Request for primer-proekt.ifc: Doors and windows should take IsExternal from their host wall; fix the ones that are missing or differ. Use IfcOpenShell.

First a look at what the model holds.

```python
import ifcopenshell
import ifcopenshell.util.element

model = ifcopenshell.open("primer-proekt.ifc")
print(model.schema)
seen = {}
for e in model.by_type("IfcDoor") + model.by_type("IfcWindow"):
    if not e.FillsVoids:
        continue
    host = e.FillsVoids[0].RelatingOpeningElement.VoidsElements[0].RelatingBuildingElement
    own = ifcopenshell.util.element.get_pset(e, f"Pset_{e.is_a()[3:].removesuffix('StandardCase')}Common", "IsExternal")
    wall = ifcopenshell.util.element.get_pset(host, "Pset_WallCommon", "IsExternal")
    seen[e.is_a(), own, wall] = seen.get((e.is_a(), own, wall), 0) + 1
for (cls, own, wall), count in sorted(seen.items(), key=str):
    print(count, cls, "IsExternal:", own, "| host wall:", wall)
```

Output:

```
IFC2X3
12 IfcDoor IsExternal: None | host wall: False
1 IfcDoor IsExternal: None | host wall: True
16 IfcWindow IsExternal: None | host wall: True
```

```python
import ifcopenshell
import ifcopenshell.api.pset
import ifcopenshell.util.element

model = ifcopenshell.open("primer-proekt.ifc")

count = 0
for ifc_class, pset_name in (("IfcDoor", "Pset_DoorCommon"), ("IfcWindow", "Pset_WindowCommon")):
    for e in model.by_type(ifc_class):
        if not e.FillsVoids:
            continue
        host = e.FillsVoids[0].RelatingOpeningElement.VoidsElements[0].RelatingBuildingElement
        external = ifcopenshell.util.element.get_pset(host, "Pset_WallCommon", "IsExternal")
        if external is None or ifcopenshell.util.element.get_pset(e, pset_name, "IsExternal") == external:
            continue
        pset = ifcopenshell.api.pset.add_pset(model, product=e, name=pset_name)
        ifcopenshell.api.pset.edit_pset(model, pset=pset, properties={"IsExternal": external})
        count += 1

print(count, "updated")

model.write("primer-proekt-out.ifc")
```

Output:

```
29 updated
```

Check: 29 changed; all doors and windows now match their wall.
